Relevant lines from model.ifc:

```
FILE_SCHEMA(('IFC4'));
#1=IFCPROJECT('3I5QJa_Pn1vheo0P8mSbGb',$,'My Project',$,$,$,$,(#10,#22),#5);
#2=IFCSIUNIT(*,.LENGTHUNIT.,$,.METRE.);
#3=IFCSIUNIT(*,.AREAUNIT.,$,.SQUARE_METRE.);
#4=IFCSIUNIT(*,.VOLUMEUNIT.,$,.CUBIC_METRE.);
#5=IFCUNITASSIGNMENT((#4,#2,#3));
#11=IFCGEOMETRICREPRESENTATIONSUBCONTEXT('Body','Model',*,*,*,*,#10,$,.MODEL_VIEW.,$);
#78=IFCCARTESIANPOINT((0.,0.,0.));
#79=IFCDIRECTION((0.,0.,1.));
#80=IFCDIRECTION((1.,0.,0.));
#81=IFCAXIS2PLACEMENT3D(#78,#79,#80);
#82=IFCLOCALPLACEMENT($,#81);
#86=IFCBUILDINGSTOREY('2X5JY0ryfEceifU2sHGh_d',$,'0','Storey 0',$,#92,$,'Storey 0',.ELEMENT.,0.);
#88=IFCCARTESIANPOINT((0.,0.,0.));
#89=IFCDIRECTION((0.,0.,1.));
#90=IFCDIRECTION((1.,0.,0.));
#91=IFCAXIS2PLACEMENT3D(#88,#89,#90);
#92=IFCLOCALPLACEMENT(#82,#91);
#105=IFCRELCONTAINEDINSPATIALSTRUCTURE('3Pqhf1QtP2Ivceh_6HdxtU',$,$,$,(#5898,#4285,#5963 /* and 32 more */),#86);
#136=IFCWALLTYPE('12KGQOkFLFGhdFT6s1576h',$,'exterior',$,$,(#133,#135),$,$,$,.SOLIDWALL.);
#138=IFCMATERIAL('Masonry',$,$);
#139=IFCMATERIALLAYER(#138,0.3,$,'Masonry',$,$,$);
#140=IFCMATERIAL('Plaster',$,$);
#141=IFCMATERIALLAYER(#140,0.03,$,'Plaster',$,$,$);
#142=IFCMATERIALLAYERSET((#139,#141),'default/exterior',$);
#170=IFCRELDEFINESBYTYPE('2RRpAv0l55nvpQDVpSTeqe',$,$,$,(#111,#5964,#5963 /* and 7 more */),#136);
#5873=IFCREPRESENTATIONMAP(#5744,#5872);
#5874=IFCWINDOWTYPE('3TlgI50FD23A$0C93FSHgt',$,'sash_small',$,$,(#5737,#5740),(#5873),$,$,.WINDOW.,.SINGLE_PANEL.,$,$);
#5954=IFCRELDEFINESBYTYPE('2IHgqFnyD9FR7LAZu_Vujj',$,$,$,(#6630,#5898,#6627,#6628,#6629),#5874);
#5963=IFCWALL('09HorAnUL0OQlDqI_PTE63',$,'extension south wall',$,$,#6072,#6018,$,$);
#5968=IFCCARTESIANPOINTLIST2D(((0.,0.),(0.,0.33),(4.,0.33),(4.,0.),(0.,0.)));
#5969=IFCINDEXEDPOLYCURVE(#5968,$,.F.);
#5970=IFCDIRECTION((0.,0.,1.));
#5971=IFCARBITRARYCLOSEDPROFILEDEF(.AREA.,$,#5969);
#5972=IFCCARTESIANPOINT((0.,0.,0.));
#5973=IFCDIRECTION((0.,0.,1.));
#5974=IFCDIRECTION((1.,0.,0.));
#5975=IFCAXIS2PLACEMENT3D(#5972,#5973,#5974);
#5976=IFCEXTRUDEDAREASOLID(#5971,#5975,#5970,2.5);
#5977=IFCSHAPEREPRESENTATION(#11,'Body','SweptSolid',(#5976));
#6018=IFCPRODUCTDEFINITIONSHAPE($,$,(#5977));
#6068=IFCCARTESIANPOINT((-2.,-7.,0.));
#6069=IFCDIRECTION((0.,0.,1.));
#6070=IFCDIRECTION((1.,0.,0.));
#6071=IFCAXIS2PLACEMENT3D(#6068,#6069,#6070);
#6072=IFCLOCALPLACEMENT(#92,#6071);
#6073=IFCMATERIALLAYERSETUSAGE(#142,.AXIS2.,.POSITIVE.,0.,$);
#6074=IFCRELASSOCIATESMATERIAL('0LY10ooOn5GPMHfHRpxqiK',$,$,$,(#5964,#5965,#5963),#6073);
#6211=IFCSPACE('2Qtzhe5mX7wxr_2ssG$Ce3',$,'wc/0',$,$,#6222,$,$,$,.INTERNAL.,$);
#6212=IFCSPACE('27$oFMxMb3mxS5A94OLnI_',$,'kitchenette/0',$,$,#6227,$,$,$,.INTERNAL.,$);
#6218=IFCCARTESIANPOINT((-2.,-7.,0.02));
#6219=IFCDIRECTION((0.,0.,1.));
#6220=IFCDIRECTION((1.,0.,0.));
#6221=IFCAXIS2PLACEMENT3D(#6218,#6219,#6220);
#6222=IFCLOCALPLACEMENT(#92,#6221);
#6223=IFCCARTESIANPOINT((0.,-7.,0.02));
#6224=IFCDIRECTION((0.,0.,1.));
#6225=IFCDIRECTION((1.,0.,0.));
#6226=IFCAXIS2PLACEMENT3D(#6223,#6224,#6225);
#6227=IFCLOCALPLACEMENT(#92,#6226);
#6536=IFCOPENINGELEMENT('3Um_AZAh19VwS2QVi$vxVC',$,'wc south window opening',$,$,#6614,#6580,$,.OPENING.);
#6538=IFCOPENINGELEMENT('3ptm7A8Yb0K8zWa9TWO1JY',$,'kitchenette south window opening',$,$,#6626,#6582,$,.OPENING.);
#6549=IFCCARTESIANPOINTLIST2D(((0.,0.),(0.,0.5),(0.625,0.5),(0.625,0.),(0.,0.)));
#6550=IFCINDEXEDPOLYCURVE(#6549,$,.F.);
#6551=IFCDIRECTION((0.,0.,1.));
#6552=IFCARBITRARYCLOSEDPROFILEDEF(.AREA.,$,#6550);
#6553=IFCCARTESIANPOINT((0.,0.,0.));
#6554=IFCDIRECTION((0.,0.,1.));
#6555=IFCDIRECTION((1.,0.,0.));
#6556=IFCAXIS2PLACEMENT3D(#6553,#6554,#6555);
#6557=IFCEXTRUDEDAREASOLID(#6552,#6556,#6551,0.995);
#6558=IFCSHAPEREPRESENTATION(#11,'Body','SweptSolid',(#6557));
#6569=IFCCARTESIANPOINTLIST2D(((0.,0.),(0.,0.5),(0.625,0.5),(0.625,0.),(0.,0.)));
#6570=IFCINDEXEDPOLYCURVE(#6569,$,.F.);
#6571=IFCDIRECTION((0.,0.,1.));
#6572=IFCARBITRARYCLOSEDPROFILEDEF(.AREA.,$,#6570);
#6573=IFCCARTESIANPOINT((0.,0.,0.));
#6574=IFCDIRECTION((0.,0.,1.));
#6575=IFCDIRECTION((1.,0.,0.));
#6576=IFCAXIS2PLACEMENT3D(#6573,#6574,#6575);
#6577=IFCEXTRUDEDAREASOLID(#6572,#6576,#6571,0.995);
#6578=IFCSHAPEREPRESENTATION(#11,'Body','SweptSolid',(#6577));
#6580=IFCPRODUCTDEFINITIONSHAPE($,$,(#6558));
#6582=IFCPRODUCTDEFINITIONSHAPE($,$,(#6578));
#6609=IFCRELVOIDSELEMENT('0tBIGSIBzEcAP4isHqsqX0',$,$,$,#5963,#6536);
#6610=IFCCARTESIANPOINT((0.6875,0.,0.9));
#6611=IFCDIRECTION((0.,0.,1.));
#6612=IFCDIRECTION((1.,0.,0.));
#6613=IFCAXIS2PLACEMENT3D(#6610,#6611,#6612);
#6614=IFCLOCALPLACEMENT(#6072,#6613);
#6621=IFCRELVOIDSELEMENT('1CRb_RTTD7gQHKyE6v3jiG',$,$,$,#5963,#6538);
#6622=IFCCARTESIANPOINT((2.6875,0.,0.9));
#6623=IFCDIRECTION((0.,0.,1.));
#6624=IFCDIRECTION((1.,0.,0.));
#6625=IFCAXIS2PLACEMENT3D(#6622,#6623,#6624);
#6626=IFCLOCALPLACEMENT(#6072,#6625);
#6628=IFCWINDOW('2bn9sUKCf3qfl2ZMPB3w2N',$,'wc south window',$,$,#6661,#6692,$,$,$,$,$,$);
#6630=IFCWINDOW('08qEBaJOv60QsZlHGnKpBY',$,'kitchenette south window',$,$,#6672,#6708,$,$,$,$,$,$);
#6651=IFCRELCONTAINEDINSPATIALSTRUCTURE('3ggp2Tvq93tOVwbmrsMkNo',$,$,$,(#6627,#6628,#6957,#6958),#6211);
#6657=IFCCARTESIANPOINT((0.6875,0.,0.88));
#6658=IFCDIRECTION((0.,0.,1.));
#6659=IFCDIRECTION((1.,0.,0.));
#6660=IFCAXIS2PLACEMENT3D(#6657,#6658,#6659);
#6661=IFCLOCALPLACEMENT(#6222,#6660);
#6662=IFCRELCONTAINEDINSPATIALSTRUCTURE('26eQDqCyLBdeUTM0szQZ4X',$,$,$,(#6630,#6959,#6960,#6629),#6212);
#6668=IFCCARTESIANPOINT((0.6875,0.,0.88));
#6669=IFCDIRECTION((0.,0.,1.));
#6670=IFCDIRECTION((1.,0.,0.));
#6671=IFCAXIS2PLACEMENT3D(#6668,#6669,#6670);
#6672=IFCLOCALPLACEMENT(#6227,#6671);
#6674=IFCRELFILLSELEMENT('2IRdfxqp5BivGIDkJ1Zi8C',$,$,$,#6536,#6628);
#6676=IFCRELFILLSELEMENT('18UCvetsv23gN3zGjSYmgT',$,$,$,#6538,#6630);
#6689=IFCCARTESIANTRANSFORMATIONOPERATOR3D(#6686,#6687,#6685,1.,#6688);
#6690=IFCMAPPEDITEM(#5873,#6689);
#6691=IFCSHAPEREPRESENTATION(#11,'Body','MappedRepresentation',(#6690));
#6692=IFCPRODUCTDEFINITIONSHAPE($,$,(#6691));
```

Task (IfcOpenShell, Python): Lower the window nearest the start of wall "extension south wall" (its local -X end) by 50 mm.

```python
import numpy as np
import ifcopenshell
import ifcopenshell.api.geometry
import ifcopenshell.util.placement
import ifcopenshell.util.unit

model = ifcopenshell.open("model.ifc")
unit_scale = ifcopenshell.util.unit.calculate_unit_scale(model)

window = model.by_id(6628)
opening = window.FillsVoids[0].RelatingOpeningElement
dz = -0.05 / unit_scale

shift = np.array([0.0, 0.0, dz])
# The window is not placed relative to its opening, so move both.
for product in (opening, window):
    matrix = ifcopenshell.util.placement.get_local_placement(product.ObjectPlacement)
    matrix[:3, 3] += shift
    ifcopenshell.api.geometry.edit_object_placement(model, product=product, matrix=matrix, is_si=False)

print(f"moved by {dz * unit_scale:+.3f} m")

model.write("model-out.ifc")
```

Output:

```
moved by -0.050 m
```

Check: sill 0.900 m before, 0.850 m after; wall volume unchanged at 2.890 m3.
